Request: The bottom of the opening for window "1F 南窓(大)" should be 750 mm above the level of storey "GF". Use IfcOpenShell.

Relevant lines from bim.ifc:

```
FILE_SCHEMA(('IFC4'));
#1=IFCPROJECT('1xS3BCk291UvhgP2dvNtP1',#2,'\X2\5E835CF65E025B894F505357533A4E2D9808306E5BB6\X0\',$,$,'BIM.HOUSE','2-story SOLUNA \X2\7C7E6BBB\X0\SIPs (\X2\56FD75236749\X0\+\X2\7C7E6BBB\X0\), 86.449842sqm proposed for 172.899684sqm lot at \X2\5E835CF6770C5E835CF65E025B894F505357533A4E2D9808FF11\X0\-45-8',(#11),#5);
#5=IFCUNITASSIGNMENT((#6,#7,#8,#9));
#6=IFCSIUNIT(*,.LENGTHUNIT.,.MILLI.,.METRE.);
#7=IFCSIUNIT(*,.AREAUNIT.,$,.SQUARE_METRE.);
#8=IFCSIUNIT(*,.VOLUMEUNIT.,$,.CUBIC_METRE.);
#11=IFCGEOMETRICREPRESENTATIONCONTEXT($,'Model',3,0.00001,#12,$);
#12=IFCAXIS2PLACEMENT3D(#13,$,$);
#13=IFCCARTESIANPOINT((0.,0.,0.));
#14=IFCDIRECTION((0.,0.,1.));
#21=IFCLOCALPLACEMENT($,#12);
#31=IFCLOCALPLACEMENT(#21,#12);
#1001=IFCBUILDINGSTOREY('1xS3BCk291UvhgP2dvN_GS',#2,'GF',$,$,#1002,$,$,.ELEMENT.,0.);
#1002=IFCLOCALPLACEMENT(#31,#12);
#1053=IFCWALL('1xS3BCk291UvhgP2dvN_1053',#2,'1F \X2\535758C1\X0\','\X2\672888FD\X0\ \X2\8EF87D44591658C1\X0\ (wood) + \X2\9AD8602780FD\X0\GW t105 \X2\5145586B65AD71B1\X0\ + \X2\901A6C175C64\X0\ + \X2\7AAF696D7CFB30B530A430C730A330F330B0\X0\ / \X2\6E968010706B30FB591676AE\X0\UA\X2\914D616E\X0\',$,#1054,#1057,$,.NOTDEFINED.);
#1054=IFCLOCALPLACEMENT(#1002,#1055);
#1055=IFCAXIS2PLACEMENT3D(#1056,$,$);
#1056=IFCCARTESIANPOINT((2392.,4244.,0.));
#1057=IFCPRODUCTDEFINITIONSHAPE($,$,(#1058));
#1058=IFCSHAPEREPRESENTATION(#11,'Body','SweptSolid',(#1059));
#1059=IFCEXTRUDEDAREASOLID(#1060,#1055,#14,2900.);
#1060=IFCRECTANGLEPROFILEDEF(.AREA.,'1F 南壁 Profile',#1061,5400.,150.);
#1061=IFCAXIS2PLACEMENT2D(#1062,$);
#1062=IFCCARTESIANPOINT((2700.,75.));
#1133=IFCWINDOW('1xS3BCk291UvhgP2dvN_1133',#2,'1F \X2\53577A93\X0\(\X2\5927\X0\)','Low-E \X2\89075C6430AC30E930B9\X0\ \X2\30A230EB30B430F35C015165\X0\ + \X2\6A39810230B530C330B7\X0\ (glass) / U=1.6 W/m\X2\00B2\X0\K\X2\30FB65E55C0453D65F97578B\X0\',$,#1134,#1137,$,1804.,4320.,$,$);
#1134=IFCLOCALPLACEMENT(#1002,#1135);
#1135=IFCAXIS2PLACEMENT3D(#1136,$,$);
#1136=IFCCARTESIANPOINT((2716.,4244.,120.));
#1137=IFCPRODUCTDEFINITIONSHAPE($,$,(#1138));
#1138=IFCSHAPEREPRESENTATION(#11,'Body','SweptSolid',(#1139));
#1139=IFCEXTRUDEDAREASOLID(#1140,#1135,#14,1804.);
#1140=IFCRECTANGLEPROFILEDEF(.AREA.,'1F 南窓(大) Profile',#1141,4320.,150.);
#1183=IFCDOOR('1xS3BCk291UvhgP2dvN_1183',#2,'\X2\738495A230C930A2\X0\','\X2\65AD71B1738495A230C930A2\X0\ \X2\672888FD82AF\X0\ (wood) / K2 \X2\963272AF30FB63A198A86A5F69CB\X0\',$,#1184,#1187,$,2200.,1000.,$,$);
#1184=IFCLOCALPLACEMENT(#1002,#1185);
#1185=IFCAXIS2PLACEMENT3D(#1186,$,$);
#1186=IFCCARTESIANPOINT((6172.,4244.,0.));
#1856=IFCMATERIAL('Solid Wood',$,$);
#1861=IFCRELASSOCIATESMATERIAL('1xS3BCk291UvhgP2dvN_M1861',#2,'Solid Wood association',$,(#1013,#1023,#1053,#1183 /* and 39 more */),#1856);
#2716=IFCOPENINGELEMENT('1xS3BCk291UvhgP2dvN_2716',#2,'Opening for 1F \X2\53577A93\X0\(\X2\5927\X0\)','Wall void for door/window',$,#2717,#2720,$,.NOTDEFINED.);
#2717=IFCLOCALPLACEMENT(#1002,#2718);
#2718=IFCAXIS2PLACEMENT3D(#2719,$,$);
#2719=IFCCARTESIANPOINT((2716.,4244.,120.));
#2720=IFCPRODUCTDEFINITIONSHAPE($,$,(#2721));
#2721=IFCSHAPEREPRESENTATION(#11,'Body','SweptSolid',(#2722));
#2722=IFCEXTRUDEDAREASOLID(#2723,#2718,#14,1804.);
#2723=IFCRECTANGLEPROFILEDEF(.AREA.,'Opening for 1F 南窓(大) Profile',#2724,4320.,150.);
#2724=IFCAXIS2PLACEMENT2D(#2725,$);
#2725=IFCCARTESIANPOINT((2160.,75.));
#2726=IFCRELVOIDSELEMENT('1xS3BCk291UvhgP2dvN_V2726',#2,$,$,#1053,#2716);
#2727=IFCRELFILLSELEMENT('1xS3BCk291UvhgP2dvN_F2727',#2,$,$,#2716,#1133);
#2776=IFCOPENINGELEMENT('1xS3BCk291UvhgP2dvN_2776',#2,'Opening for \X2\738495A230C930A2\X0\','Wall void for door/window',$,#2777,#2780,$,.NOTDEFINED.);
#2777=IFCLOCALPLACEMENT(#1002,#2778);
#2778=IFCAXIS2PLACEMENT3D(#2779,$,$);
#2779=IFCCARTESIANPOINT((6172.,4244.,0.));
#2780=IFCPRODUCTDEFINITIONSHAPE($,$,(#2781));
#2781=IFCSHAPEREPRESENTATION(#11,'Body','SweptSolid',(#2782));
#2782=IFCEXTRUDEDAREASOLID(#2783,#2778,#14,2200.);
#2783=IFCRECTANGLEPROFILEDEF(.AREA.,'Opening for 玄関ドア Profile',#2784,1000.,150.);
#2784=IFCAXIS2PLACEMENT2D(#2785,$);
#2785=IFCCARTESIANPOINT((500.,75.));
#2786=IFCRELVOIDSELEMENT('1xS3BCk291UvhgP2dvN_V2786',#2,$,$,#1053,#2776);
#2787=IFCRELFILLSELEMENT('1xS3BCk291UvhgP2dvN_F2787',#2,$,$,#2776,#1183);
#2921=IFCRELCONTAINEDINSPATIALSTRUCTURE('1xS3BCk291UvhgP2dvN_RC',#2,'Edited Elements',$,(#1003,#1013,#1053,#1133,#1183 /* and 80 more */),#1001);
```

```python
import numpy as np
import ifcopenshell
import ifcopenshell.api.geometry
import ifcopenshell.geom
import ifcopenshell.util.element
import ifcopenshell.util.placement
import ifcopenshell.util.shape
import ifcopenshell.util.unit

model = ifcopenshell.open("bim.ifc")
unit_scale = ifcopenshell.util.unit.calculate_unit_scale(model)

window = model.by_guid("1xS3BCk291UvhgP2dvN_1133")
opening = window.FillsVoids[0].RelatingOpeningElement
storey = ifcopenshell.util.element.get_container(window, ifc_class="IfcBuildingStorey")
level = ifcopenshell.util.placement.get_local_placement(storey.ObjectPlacement)[2, 3]

# The opening's origin need not be at the sill, so measure its lowest point.
shape = ifcopenshell.geom.create_shape(ifcopenshell.geom.settings(), opening)
bottom = ifcopenshell.util.shape.get_shape_bottom_elevation(shape, shape.geometry) / unit_scale
dz = level + 0.75 / unit_scale - bottom

shift = np.array([0.0, 0.0, dz])
# The window is not placed relative to its opening, so move both.
for product in (opening, window):
    matrix = ifcopenshell.util.placement.get_local_placement(product.ObjectPlacement)
    matrix[:3, 3] += shift
    ifcopenshell.api.geometry.edit_object_placement(model, product=product, matrix=matrix, is_si=False)

print(f"moved by {dz * unit_scale:+.3f} m")

model.write("bim_updated.ifc")
```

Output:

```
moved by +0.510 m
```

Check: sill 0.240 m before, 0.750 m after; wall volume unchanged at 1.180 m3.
